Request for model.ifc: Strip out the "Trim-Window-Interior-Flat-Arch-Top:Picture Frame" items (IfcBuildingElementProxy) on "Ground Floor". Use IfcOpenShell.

First a look at what the model holds.

```python
import ifcopenshell
import ifcopenshell.util.element

model = ifcopenshell.open("model.ifc")
print(model.schema)
storey = next(s for s in model.by_type("IfcBuildingStorey") if s.Name == "Ground Floor")
proxies = [e for e in ifcopenshell.util.element.get_decomposition(storey) if e.is_a("IfcBuildingElementProxy")]
seen = {}
for e in proxies:
    element_type = ifcopenshell.util.element.get_type(e)
    name = element_type.Name if element_type not in (None, e) else None
    seen[name] = seen.get(name, 0) + 1
for name, count in sorted(seen.items(), key=str):
    print(count, "x", name)
```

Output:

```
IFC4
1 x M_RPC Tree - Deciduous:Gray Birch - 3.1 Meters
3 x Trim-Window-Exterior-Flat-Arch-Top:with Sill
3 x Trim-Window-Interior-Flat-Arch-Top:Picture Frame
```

```python
import ifcopenshell
import ifcopenshell.api.root
import ifcopenshell.util.element

model = ifcopenshell.open("model.ifc")

storey = next(s for s in model.by_type("IfcBuildingStorey") if s.Name == "Ground Floor")
proxies = [e for e in ifcopenshell.util.element.get_decomposition(storey) if e.is_a("IfcBuildingElementProxy")]
targets = [e for e in proxies if (t := ifcopenshell.util.element.get_type(e)) not in (None, e) and t.Name == "Trim-Window-Interior-Flat-Arch-Top:Picture Frame"]

for e in targets:
    ifcopenshell.api.root.remove_product(model, product=e)
print(len(targets), "removed")

model.write("model_edited.ifc")
```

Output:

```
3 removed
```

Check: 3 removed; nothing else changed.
